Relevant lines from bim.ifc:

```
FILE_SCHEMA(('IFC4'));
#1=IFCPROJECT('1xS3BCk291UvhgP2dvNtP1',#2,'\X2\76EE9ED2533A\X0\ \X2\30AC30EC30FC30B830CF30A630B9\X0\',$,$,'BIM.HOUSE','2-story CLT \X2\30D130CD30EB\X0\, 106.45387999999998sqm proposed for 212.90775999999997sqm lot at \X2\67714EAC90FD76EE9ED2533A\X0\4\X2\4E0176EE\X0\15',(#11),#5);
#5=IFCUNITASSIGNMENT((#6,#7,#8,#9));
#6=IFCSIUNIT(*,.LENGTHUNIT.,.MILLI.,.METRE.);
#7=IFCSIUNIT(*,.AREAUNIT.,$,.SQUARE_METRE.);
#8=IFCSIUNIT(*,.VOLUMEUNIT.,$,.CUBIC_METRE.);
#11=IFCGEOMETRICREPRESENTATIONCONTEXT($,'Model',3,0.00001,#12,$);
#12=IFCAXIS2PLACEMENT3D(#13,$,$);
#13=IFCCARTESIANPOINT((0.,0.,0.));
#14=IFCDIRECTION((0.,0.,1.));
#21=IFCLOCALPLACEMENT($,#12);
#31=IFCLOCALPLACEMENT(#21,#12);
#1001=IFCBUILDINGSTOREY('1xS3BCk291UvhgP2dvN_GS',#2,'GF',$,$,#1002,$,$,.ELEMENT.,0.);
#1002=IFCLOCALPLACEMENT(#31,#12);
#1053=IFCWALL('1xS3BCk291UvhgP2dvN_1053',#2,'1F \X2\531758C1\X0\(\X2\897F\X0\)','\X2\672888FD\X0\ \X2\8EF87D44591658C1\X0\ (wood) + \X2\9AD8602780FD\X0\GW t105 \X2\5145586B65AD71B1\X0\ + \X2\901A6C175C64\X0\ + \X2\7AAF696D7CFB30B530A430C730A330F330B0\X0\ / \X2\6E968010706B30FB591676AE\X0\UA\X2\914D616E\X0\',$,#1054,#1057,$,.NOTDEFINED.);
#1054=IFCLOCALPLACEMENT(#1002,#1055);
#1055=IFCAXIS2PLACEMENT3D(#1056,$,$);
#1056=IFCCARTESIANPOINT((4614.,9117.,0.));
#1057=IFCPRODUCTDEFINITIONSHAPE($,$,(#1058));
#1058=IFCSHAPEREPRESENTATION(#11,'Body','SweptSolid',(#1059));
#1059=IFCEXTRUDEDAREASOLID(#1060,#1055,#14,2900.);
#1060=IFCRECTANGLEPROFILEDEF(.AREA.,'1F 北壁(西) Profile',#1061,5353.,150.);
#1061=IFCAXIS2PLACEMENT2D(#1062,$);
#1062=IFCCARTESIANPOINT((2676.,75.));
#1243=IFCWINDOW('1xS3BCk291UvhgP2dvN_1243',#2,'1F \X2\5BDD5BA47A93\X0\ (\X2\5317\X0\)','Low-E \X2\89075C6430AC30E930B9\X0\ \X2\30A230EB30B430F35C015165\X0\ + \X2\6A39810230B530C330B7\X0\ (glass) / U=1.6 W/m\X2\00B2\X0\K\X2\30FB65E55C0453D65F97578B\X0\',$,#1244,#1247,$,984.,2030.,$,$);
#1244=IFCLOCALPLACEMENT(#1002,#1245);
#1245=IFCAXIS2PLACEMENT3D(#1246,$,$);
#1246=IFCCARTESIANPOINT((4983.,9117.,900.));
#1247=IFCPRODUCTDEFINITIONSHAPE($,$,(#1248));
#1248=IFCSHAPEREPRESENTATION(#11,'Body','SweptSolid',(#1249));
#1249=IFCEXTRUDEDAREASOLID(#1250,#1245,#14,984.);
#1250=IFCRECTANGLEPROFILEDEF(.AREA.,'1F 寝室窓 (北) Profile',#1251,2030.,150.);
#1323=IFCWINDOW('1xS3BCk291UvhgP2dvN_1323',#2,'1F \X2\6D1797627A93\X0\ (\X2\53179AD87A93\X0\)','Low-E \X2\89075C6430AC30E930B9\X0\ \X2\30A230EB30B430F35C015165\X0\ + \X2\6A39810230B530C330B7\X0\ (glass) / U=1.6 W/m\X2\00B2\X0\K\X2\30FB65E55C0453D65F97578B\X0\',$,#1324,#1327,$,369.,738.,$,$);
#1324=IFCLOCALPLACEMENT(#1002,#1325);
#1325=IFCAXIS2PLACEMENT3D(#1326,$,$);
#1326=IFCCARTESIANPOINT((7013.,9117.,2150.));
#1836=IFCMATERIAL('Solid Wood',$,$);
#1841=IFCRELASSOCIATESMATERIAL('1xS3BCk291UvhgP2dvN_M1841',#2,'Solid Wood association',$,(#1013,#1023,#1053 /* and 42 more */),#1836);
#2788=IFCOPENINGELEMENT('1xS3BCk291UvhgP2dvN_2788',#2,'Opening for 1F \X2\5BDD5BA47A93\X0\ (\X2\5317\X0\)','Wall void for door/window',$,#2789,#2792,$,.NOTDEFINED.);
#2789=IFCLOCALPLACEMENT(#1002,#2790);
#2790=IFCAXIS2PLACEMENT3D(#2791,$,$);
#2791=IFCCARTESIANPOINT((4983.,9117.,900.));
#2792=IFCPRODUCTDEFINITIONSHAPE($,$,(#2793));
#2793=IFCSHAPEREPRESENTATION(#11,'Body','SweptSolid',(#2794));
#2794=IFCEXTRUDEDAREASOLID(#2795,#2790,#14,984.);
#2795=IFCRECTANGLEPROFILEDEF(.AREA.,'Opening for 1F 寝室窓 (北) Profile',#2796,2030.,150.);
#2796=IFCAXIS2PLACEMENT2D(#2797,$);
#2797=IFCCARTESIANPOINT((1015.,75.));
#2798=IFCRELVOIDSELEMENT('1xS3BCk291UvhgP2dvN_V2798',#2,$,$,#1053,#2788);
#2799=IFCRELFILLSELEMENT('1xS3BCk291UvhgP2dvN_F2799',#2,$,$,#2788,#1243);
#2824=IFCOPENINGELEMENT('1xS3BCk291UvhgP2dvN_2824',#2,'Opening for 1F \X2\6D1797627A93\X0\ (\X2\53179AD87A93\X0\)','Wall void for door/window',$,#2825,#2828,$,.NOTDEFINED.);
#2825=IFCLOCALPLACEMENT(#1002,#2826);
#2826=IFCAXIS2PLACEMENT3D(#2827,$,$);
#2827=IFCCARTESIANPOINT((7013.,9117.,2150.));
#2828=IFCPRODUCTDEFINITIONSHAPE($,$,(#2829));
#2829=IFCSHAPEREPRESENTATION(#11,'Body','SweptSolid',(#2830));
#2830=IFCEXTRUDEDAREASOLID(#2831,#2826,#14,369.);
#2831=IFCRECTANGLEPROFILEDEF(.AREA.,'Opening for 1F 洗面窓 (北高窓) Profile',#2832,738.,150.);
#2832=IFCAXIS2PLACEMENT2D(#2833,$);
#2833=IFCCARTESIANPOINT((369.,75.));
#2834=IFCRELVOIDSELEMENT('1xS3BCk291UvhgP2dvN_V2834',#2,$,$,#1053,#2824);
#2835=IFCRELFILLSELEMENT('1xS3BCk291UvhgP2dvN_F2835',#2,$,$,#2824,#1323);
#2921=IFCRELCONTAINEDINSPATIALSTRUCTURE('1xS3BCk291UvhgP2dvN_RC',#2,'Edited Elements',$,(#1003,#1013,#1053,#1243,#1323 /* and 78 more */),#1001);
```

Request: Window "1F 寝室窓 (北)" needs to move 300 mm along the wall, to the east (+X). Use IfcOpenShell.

```python
import ifcopenshell
import ifcopenshell.api.geometry
import ifcopenshell.util.placement

model = ifcopenshell.open("bim.ifc")

window = model.by_guid("1xS3BCk291UvhgP2dvN_1243")
opening = window.FillsVoids[0].RelatingOpeningElement
wall = opening.VoidsElements[0].RelatingBuildingElement

wall_matrix = ifcopenshell.util.placement.get_local_placement(wall.ObjectPlacement)
shift = wall_matrix[:3, 0] * 300.0
before = ifcopenshell.util.placement.get_local_placement(window.ObjectPlacement)[:3, 3].copy()

# The window is not placed relative to its opening, so move both.
for product in (opening, window):
    matrix = ifcopenshell.util.placement.get_local_placement(product.ObjectPlacement)
    matrix[:3, 3] += shift
    ifcopenshell.api.geometry.edit_object_placement(model, product=product, matrix=matrix, is_si=False)

after = ifcopenshell.util.placement.get_local_placement(window.ObjectPlacement)[:3, 3]
print("window moved by", (after - before).round(3) + 0.0)

model.write("bim-out.ifc")
```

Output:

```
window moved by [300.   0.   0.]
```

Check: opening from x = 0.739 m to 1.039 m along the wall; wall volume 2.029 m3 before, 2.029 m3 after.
